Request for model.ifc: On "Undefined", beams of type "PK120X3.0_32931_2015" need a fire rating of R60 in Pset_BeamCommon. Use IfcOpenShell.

First a look at what the model holds.

```python
import ifcopenshell
import ifcopenshell.util.element

model = ifcopenshell.open("model.ifc")
print(model.schema)
storey = next(s for s in model.by_type("IfcBuildingStorey") if s.Name == "Undefined")
beams = [e for e in ifcopenshell.util.element.get_decomposition(storey) if e.is_a("IfcBeam")]
seen = {}
for e in beams:
    element_type = ifcopenshell.util.element.get_type(e)
    key = (element_type.Name if element_type != e and element_type else None, ifcopenshell.util.element.get_pset(e, "Pset_BeamCommon", "FireRating"))
    seen[key] = seen.get(key, 0) + 1
for (name, value), count in sorted(seen.items(), key=str):
    print(count, "x", name, "|", value)
```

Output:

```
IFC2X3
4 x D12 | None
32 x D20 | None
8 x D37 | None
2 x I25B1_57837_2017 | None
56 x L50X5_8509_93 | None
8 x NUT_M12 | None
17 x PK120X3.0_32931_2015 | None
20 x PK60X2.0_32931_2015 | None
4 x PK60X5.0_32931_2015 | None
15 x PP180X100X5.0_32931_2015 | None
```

```python
import ifcopenshell
import ifcopenshell.api.pset
import ifcopenshell.util.element

model = ifcopenshell.open("model.ifc")

storey = next(s for s in model.by_type("IfcBuildingStorey") if s.Name == "Undefined")
beams = [e for e in ifcopenshell.util.element.get_decomposition(storey) if e.is_a("IfcBeam")]

count = 0
for e in beams:
    element_type = ifcopenshell.util.element.get_type(e)
    if element_type in (None, e) or element_type.Name != "PK120X3.0_32931_2015":
        continue
    found = ifcopenshell.util.element.get_pset(e, "Pset_BeamCommon", should_inherit=False)
    if found:
        pset = model.by_id(found["id"])
        if len(ifcopenshell.util.element.get_elements_by_pset(pset)) > 1:
            pset = ifcopenshell.api.pset.unshare_pset(model, products=[e], pset=pset)[0]
    else:
        pset = ifcopenshell.api.pset.add_pset(model, product=e, name="Pset_BeamCommon")
    ifcopenshell.api.pset.edit_pset(model, pset=pset, properties={"FireRating": "R60"})
    count += 1

print(count, "beams updated")

model.write("model_v2.ifc")
```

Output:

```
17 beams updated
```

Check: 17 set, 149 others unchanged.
